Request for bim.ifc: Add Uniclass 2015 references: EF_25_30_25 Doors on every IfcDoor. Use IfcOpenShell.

First a look at what the model holds.

```python
import ifcopenshell

model = ifcopenshell.open("bim.ifc")
print(model.schema)
print("classifications:", [c.Name for c in model.by_type("IfcClassification")])
for ifc_class in ("IfcDoor", "IfcRoof", "IfcStair", "IfcWall", "IfcWindow"):
    print(ifc_class, len(model.by_type(ifc_class)))
```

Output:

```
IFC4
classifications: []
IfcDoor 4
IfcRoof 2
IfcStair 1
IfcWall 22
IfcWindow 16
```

```python
import ifcopenshell
import ifcopenshell.api.classification

model = ifcopenshell.open("bim.ifc")

system = ifcopenshell.api.classification.add_classification(model, classification="Uniclass 2015")

codes = {
    "IfcDoor": ("EF_25_30_25", "Doors"),
}
for ifc_class, (code, name) in codes.items():
    products = model.by_type(ifc_class)
    ifcopenshell.api.classification.add_reference(
        model, products=products, classification=system, identification=code, name=name
    )
    print(code, len(products))

model.write("bim_rev.ifc")
```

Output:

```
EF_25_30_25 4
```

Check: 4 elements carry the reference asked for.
